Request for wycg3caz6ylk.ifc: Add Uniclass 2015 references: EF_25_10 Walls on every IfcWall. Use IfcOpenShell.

First a look at what the model holds.

```python
import ifcopenshell

model = ifcopenshell.open("wycg3caz6ylk.ifc")
print(model.schema)
print("classifications:", [c.Name for c in model.by_type("IfcClassification")])
for ifc_class in ("IfcDoor", "IfcRoof", "IfcStair", "IfcWall", "IfcWindow"):
    print(ifc_class, len(model.by_type(ifc_class)))
```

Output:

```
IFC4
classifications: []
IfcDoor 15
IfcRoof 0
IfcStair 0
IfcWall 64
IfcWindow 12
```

```python
import ifcopenshell
import ifcopenshell.api.classification

model = ifcopenshell.open("wycg3caz6ylk.ifc")

system = ifcopenshell.api.classification.add_classification(model, classification="Uniclass 2015")

codes = {
    "IfcWall": ("EF_25_10", "Walls"),
}
for ifc_class, (code, name) in codes.items():
    products = model.by_type(ifc_class)
    ifcopenshell.api.classification.add_reference(
        model, products=products, classification=system, identification=code, name=name
    )
    print(code, len(products))

model.write("wycg3caz6ylk-out.ifc")
```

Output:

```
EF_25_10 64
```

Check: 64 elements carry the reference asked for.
